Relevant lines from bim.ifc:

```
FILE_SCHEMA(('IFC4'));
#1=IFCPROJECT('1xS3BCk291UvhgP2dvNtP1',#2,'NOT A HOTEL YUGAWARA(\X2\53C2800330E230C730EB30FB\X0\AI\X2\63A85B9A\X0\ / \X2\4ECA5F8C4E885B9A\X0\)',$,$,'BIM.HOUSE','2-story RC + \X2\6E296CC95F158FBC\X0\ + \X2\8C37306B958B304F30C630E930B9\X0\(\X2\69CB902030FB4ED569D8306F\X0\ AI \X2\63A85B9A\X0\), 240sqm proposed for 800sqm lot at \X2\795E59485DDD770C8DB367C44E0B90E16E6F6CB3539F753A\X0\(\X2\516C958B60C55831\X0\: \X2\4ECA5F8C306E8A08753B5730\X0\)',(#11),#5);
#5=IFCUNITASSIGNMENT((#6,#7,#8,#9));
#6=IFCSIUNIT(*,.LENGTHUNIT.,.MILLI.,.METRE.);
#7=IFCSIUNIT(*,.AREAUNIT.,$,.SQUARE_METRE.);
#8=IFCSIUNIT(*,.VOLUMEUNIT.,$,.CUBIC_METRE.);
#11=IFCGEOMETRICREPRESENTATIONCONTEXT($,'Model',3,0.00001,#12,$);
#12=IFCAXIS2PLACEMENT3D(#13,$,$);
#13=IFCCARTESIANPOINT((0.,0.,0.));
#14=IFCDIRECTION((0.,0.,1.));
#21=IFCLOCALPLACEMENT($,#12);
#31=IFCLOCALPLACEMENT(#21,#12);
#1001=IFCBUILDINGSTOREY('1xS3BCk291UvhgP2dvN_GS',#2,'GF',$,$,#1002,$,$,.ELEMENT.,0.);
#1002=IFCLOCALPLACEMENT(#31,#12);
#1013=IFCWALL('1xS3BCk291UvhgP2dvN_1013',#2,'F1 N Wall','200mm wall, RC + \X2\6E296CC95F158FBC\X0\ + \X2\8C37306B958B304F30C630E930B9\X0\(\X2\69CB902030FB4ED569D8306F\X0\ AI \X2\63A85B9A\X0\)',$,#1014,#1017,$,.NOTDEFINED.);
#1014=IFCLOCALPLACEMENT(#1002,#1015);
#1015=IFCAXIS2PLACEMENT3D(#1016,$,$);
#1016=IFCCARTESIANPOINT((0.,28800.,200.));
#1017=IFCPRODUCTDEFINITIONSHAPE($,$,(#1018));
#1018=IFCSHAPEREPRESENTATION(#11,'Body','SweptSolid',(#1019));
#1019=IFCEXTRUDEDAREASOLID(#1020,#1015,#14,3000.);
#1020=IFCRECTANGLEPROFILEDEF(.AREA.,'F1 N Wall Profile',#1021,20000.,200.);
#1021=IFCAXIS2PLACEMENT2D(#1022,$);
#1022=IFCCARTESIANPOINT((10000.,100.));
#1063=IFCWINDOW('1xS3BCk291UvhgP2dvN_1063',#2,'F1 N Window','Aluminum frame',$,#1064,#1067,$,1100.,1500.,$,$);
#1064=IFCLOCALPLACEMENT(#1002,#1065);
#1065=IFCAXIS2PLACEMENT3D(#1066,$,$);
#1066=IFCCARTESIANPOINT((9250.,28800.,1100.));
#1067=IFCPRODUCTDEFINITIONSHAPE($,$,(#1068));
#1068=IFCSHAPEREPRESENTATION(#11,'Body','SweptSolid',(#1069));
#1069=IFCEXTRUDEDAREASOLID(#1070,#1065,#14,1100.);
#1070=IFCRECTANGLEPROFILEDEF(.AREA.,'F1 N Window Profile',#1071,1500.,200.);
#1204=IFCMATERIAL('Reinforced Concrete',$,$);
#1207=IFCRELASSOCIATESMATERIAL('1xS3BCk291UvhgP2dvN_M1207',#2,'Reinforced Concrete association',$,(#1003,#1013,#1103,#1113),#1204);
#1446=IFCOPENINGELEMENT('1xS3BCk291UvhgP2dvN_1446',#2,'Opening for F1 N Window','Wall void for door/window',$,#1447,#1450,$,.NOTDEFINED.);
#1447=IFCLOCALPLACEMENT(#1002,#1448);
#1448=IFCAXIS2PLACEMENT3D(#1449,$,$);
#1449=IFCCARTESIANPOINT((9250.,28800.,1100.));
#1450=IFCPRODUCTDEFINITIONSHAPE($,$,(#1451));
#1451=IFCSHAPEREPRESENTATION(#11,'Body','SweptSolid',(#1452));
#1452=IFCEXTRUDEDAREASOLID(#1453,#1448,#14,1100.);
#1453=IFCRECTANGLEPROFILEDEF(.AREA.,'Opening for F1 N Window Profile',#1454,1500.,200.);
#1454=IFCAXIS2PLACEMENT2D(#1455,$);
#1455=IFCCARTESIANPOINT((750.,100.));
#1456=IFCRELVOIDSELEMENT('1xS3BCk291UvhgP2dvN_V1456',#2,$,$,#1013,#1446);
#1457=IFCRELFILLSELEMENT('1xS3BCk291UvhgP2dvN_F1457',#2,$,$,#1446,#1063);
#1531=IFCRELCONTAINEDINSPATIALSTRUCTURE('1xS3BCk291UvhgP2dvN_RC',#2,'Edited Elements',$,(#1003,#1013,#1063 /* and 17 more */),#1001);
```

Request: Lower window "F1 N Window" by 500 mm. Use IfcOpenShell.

```python
import numpy as np
import ifcopenshell
import ifcopenshell.api.geometry
import ifcopenshell.util.placement
import ifcopenshell.util.unit

model = ifcopenshell.open("bim.ifc")
unit_scale = ifcopenshell.util.unit.calculate_unit_scale(model)

window = model.by_guid("1xS3BCk291UvhgP2dvN_1063")
opening = window.FillsVoids[0].RelatingOpeningElement
dz = -0.5 / unit_scale

shift = np.array([0.0, 0.0, dz])
# The window is not placed relative to its opening, so move both.
for product in (opening, window):
    matrix = ifcopenshell.util.placement.get_local_placement(product.ObjectPlacement)
    matrix[:3, 3] += shift
    ifcopenshell.api.geometry.edit_object_placement(model, product=product, matrix=matrix, is_si=False)

print(f"moved by {dz * unit_scale:+.3f} m")

model.write("bim_updated.ifc")
```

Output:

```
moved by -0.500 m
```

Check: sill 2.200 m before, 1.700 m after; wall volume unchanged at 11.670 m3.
